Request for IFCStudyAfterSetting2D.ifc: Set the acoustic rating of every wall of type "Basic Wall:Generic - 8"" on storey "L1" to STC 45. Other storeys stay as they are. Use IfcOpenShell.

First a look at what the model holds.

```python
import ifcopenshell
import ifcopenshell.util.element

model = ifcopenshell.open("IFCStudyAfterSetting2D.ifc")
print(model.schema)
storey = next(s for s in model.by_type("IfcBuildingStorey") if s.Name == "L1")
walls = [e for e in ifcopenshell.util.element.get_decomposition(storey) if e.is_a("IfcWall")]
seen = {}
for e in walls:
    element_type = ifcopenshell.util.element.get_type(e)
    key = (element_type.Name if element_type != e and element_type else None, ifcopenshell.util.element.get_pset(e, "Pset_WallCommon", "AcousticRating"))
    seen[key] = seen.get(key, 0) + 1
for (name, value), count in sorted(seen.items(), key=str):
    print(count, "x", name, "|", value)
```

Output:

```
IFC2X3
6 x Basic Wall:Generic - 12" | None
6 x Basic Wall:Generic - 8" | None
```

```python
import ifcopenshell
import ifcopenshell.api.pset
import ifcopenshell.util.element

model = ifcopenshell.open("IFCStudyAfterSetting2D.ifc")

storey = next(s for s in model.by_type("IfcBuildingStorey") if s.Name == "L1")
walls = [e for e in ifcopenshell.util.element.get_decomposition(storey) if e.is_a("IfcWall")]

count = 0
for e in walls:
    element_type = ifcopenshell.util.element.get_type(e)
    if element_type in (None, e) or element_type.Name != 'Basic Wall:Generic - 8"':
        continue
    # add_pset returns the element's existing set when there is one.
    pset = ifcopenshell.api.pset.add_pset(model, product=e, name="Pset_WallCommon")
    ifcopenshell.api.pset.edit_pset(model, pset=pset, properties={"AcousticRating": "STC 45"})
    count += 1

print(count, "walls updated")

model.write("IFCStudyAfterSetting2D_edited.ifc")
```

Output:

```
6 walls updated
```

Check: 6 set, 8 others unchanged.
